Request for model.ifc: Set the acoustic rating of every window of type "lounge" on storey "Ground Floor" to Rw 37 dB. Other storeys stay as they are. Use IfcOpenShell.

First a look at what the model holds.

```python
import ifcopenshell
import ifcopenshell.util.element

model = ifcopenshell.open("model.ifc")
print(model.schema)
storey = next(s for s in model.by_type("IfcBuildingStorey") if s.Name == "Ground Floor")
windows = [e for e in ifcopenshell.util.element.get_decomposition(storey) if e.is_a("IfcWindow")]
seen = {}
for e in windows:
    element_type = ifcopenshell.util.element.get_type(e)
    key = (element_type.Name if element_type != e and element_type else None, ifcopenshell.util.element.get_pset(e, "Pset_WindowCommon", "AcousticRating"))
    seen[key] = seen.get(key, 0) + 1
for (name, value), count in sorted(seen.items(), key=str):
    print(count, "x", name, "|", value)
```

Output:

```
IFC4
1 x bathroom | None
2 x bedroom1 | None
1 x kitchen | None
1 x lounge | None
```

```python
import ifcopenshell
import ifcopenshell.api.pset
import ifcopenshell.util.element

model = ifcopenshell.open("model.ifc")

storey = next(s for s in model.by_type("IfcBuildingStorey") if s.Name == "Ground Floor")
windows = [e for e in ifcopenshell.util.element.get_decomposition(storey) if e.is_a("IfcWindow")]

count = 0
for e in windows:
    element_type = ifcopenshell.util.element.get_type(e)
    if element_type in (None, e) or element_type.Name != "lounge":
        continue
    # add_pset returns the element's existing set when there is one.
    pset = ifcopenshell.api.pset.add_pset(model, product=e, name="Pset_WindowCommon")
    ifcopenshell.api.pset.edit_pset(model, pset=pset, properties={"AcousticRating": "Rw 37 dB"})
    count += 1

print(count, "windows updated")

model.write("model_v2.ifc")
```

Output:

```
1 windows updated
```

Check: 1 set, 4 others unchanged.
